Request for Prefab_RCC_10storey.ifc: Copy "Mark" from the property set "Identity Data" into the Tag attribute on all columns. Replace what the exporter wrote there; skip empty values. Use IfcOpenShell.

First a look at what the model holds.

```python
import ifcopenshell
import ifcopenshell.util.element

model = ifcopenshell.open("Prefab_RCC_10storey.ifc")
print(model.schema)
columns = model.by_type("IfcColumn")
print(len(columns), "columns")
for e in columns[:8]:
    source = ifcopenshell.util.element.get_pset(e, "Identity Data", "Mark")
    target = e.Tag
    print(e.id(), repr(source), repr(target), sep=" | ")
```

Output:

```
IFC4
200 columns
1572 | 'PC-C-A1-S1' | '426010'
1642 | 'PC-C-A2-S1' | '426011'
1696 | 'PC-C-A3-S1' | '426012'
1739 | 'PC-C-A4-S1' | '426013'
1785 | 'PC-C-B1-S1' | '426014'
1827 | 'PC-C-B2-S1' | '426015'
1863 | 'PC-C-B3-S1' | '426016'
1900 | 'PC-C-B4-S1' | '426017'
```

```python
import ifcopenshell
import ifcopenshell.util.element

model = ifcopenshell.open("Prefab_RCC_10storey.ifc")

count = 0
for e in model.by_type("IfcColumn"):
    value = ifcopenshell.util.element.get_pset(e, "Identity Data", "Mark")
    current = e.Tag
    if not value or not value.strip() or current == value:
        continue
    e.Tag = value
    count += 1

print(count, "columns updated")

model.write("Prefab_RCC_10storey_rev.ifc")
```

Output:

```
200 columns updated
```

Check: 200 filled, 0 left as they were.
